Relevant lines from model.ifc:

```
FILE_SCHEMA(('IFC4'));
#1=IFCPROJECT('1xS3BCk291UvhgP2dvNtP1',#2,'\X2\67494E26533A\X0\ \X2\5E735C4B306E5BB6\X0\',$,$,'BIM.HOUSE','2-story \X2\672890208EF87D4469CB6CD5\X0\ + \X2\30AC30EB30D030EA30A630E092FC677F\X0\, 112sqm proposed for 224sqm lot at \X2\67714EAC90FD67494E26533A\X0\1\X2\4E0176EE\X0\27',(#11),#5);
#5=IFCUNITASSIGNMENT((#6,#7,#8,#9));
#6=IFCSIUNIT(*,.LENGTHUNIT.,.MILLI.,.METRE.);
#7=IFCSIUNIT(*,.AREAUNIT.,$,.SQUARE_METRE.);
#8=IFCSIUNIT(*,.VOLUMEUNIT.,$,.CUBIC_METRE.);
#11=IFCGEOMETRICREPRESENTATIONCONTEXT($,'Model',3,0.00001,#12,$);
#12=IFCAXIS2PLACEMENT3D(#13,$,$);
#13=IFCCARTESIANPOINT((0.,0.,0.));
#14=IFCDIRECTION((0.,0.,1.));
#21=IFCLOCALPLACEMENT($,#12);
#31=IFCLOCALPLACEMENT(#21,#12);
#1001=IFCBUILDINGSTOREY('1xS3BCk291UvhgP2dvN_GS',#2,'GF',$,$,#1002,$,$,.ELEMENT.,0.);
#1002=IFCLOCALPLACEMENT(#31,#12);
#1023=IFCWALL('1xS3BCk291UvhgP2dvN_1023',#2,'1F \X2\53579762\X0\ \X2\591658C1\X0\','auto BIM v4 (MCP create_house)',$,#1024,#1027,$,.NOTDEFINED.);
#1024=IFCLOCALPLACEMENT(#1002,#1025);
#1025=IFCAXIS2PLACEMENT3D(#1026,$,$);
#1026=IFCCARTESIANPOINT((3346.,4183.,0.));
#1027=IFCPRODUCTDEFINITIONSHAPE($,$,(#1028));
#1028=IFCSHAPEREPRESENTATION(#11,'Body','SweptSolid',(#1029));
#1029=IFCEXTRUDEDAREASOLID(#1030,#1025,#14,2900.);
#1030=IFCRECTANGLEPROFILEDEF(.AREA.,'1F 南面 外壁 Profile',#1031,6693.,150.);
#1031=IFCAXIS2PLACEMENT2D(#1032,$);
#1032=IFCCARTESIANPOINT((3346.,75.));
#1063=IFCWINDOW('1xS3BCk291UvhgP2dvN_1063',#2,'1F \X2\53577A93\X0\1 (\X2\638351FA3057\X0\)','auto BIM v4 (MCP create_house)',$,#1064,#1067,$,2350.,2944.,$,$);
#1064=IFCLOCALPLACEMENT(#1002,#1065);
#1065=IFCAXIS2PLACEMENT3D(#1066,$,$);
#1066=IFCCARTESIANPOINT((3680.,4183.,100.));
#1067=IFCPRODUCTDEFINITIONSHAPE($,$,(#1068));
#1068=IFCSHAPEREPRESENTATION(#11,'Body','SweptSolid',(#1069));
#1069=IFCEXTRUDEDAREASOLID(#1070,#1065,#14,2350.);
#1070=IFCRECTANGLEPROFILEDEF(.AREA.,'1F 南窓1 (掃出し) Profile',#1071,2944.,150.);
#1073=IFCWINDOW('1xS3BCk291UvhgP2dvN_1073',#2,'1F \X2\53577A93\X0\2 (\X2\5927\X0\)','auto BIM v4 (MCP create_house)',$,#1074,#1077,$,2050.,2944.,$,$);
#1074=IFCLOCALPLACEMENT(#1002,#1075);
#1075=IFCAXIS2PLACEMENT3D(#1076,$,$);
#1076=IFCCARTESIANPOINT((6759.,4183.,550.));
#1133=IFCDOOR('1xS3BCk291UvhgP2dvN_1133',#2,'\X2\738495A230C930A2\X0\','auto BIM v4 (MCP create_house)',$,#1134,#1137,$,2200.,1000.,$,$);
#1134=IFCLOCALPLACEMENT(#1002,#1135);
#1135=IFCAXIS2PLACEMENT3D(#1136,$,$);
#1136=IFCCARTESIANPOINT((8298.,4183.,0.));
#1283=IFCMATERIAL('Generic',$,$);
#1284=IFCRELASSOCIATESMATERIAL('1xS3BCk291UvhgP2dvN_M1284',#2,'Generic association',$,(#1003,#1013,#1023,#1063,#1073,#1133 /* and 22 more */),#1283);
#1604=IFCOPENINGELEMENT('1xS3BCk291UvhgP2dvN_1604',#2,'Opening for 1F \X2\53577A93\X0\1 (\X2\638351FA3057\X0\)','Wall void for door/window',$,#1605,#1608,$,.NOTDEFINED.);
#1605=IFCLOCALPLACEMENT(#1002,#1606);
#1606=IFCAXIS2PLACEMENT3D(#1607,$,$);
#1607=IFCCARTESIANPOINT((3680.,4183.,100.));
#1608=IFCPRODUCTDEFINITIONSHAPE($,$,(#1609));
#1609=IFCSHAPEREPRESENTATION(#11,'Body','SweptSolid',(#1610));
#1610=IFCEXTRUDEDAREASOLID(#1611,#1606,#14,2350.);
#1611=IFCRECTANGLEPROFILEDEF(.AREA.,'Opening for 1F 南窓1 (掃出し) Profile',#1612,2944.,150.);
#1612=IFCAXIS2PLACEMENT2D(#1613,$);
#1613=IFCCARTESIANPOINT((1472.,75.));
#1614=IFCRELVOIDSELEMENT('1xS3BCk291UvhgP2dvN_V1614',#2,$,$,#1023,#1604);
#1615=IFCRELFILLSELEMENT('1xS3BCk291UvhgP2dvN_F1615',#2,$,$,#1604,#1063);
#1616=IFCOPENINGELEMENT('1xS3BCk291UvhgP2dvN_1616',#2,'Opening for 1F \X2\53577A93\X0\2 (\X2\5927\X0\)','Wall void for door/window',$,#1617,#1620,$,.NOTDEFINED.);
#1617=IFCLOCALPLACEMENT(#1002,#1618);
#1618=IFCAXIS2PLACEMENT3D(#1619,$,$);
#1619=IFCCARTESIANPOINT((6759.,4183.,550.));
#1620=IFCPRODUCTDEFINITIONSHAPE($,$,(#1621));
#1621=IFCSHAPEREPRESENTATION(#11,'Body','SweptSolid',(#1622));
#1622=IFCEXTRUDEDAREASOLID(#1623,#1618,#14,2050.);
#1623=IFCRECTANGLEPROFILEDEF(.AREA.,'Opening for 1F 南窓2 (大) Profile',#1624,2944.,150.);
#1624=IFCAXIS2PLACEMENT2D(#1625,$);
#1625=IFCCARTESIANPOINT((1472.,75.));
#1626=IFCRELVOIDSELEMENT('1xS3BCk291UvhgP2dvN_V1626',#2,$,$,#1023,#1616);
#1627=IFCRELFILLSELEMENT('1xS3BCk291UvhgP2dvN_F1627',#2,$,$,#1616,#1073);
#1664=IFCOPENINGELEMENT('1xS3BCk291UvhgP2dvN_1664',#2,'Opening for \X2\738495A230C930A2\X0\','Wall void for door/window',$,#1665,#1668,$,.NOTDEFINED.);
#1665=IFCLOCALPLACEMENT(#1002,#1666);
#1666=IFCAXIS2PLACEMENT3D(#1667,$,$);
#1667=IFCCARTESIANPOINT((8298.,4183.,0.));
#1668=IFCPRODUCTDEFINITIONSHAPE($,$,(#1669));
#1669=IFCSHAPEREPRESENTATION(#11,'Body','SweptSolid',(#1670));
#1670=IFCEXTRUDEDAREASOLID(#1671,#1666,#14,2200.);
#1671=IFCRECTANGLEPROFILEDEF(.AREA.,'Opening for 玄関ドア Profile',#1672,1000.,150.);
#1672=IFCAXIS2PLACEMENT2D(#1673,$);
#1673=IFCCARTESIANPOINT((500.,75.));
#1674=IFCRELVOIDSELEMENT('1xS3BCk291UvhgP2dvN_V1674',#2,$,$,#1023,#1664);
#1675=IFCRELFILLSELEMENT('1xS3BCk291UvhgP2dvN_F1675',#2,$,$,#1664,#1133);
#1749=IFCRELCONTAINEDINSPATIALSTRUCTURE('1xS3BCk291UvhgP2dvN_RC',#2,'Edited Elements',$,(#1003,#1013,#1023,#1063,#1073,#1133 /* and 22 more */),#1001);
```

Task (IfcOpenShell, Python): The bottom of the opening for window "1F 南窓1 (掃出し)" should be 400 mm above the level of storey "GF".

```python
import numpy as np
import ifcopenshell
import ifcopenshell.api.geometry
import ifcopenshell.geom
import ifcopenshell.util.element
import ifcopenshell.util.placement
import ifcopenshell.util.shape
import ifcopenshell.util.unit

model = ifcopenshell.open("model.ifc")
unit_scale = ifcopenshell.util.unit.calculate_unit_scale(model)

window = model.by_guid("1xS3BCk291UvhgP2dvN_1063")
opening = window.FillsVoids[0].RelatingOpeningElement
storey = ifcopenshell.util.element.get_container(window, ifc_class="IfcBuildingStorey")
level = ifcopenshell.util.placement.get_local_placement(storey.ObjectPlacement)[2, 3]

# The opening's origin need not be at the sill, so measure its lowest point.
shape = ifcopenshell.geom.create_shape(ifcopenshell.geom.settings(), opening)
bottom = ifcopenshell.util.shape.get_shape_bottom_elevation(shape, shape.geometry) / unit_scale
dz = level + 400.0 - bottom

shift = np.array([0.0, 0.0, dz])
# The window is not placed relative to its opening, so move both.
for product in (opening, window):
    matrix = ifcopenshell.util.placement.get_local_placement(product.ObjectPlacement)
    matrix[:3, 3] += shift
    ifcopenshell.api.geometry.edit_object_placement(model, product=product, matrix=matrix, is_si=False)

print(f"moved by {dz * unit_scale:+.3f} m")

model.write("model_rev.ifc")
```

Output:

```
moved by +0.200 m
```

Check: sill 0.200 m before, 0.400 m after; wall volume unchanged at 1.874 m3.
